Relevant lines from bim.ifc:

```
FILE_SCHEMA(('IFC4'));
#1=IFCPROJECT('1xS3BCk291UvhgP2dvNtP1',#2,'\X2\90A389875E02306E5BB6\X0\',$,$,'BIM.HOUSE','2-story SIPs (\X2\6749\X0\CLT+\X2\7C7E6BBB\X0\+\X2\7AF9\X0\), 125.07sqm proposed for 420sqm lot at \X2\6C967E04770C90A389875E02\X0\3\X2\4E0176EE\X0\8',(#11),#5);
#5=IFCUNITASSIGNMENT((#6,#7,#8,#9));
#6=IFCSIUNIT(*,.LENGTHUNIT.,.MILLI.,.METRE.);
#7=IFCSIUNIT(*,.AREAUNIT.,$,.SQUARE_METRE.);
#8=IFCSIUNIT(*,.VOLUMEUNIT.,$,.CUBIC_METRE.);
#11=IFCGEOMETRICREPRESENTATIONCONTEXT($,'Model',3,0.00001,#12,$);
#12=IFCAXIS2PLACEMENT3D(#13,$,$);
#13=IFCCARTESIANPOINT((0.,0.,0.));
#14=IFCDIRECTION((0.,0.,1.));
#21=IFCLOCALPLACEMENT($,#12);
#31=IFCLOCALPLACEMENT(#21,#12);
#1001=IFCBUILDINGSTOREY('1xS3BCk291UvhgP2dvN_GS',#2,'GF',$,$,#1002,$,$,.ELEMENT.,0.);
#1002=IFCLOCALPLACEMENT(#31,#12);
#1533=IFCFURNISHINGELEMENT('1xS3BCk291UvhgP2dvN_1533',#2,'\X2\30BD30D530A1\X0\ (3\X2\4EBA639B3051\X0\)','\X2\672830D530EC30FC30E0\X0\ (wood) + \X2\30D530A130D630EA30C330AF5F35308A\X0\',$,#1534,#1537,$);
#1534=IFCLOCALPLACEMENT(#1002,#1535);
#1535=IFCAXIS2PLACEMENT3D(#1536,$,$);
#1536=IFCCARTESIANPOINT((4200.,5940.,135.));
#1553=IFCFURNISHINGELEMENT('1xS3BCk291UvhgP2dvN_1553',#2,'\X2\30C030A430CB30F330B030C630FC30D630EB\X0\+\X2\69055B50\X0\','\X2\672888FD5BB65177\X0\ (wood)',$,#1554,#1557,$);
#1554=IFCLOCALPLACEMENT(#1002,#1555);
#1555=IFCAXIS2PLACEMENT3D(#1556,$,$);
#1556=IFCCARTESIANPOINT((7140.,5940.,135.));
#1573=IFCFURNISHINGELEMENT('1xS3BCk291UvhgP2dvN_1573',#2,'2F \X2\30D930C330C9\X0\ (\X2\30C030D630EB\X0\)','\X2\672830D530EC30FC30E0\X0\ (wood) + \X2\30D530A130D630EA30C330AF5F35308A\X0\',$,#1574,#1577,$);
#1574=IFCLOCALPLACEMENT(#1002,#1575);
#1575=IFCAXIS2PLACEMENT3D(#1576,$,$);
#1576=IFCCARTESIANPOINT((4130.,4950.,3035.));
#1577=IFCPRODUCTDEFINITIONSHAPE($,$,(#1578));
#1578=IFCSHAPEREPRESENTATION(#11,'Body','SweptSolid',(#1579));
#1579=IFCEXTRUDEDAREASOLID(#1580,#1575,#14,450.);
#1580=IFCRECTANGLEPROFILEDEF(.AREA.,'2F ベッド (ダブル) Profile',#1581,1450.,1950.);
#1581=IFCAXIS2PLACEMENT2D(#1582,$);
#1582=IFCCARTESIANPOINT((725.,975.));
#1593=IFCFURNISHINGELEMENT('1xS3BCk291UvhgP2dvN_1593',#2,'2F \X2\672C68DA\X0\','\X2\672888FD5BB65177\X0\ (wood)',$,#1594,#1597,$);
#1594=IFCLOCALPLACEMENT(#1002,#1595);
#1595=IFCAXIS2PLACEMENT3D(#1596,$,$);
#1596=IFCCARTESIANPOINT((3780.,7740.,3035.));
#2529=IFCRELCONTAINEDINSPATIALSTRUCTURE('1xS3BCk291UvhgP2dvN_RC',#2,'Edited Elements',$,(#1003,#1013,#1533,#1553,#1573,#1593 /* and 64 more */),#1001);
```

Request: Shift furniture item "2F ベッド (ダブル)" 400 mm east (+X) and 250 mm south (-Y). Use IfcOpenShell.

```python
import ifcopenshell
import ifcopenshell.api.geometry
import ifcopenshell.util.placement
import ifcopenshell.util.unit

model = ifcopenshell.open("bim.ifc")
unit_scale = ifcopenshell.util.unit.calculate_unit_scale(model)

item = model.by_guid("1xS3BCk291UvhgP2dvN_1573")
matrix = ifcopenshell.util.placement.get_local_placement(item.ObjectPlacement)
matrix[0, 3] += 0.4 / unit_scale
matrix[1, 3] -= 0.25 / unit_scale
ifcopenshell.api.geometry.edit_object_placement(model, product=item, matrix=matrix, is_si=False)

print(ifcopenshell.util.placement.get_local_placement(item.ObjectPlacement).round(3) + 0.0)

model.write("bim_updated.ifc")
```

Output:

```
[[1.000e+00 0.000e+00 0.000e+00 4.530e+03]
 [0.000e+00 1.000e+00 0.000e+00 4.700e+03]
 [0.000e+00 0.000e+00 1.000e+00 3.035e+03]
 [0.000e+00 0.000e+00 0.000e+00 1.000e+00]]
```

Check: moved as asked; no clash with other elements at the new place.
